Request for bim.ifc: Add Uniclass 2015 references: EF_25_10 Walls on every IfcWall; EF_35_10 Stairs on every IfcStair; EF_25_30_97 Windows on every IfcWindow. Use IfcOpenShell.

First a look at what the model holds.

```python
import ifcopenshell

model = ifcopenshell.open("bim.ifc")
print(model.schema)
print("classifications:", [c.Name for c in model.by_type("IfcClassification")])
for ifc_class in ("IfcDoor", "IfcRoof", "IfcStair", "IfcWall", "IfcWindow"):
    print(ifc_class, len(model.by_type(ifc_class)))
```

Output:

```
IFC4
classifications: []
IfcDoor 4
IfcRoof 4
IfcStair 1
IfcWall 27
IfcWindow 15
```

```python
import ifcopenshell
import ifcopenshell.api.classification

model = ifcopenshell.open("bim.ifc")

system = ifcopenshell.api.classification.add_classification(model, classification="Uniclass 2015")

codes = {
    "IfcWall": ("EF_25_10", "Walls"),
    "IfcStair": ("EF_35_10", "Stairs"),
    "IfcWindow": ("EF_25_30_97", "Windows"),
}
for ifc_class, (code, name) in codes.items():
    products = model.by_type(ifc_class)
    ifcopenshell.api.classification.add_reference(
        model, products=products, classification=system, identification=code, name=name
    )
    print(code, len(products))

model.write("bim_updated.ifc")
```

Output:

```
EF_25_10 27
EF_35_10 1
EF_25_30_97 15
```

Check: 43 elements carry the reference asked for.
